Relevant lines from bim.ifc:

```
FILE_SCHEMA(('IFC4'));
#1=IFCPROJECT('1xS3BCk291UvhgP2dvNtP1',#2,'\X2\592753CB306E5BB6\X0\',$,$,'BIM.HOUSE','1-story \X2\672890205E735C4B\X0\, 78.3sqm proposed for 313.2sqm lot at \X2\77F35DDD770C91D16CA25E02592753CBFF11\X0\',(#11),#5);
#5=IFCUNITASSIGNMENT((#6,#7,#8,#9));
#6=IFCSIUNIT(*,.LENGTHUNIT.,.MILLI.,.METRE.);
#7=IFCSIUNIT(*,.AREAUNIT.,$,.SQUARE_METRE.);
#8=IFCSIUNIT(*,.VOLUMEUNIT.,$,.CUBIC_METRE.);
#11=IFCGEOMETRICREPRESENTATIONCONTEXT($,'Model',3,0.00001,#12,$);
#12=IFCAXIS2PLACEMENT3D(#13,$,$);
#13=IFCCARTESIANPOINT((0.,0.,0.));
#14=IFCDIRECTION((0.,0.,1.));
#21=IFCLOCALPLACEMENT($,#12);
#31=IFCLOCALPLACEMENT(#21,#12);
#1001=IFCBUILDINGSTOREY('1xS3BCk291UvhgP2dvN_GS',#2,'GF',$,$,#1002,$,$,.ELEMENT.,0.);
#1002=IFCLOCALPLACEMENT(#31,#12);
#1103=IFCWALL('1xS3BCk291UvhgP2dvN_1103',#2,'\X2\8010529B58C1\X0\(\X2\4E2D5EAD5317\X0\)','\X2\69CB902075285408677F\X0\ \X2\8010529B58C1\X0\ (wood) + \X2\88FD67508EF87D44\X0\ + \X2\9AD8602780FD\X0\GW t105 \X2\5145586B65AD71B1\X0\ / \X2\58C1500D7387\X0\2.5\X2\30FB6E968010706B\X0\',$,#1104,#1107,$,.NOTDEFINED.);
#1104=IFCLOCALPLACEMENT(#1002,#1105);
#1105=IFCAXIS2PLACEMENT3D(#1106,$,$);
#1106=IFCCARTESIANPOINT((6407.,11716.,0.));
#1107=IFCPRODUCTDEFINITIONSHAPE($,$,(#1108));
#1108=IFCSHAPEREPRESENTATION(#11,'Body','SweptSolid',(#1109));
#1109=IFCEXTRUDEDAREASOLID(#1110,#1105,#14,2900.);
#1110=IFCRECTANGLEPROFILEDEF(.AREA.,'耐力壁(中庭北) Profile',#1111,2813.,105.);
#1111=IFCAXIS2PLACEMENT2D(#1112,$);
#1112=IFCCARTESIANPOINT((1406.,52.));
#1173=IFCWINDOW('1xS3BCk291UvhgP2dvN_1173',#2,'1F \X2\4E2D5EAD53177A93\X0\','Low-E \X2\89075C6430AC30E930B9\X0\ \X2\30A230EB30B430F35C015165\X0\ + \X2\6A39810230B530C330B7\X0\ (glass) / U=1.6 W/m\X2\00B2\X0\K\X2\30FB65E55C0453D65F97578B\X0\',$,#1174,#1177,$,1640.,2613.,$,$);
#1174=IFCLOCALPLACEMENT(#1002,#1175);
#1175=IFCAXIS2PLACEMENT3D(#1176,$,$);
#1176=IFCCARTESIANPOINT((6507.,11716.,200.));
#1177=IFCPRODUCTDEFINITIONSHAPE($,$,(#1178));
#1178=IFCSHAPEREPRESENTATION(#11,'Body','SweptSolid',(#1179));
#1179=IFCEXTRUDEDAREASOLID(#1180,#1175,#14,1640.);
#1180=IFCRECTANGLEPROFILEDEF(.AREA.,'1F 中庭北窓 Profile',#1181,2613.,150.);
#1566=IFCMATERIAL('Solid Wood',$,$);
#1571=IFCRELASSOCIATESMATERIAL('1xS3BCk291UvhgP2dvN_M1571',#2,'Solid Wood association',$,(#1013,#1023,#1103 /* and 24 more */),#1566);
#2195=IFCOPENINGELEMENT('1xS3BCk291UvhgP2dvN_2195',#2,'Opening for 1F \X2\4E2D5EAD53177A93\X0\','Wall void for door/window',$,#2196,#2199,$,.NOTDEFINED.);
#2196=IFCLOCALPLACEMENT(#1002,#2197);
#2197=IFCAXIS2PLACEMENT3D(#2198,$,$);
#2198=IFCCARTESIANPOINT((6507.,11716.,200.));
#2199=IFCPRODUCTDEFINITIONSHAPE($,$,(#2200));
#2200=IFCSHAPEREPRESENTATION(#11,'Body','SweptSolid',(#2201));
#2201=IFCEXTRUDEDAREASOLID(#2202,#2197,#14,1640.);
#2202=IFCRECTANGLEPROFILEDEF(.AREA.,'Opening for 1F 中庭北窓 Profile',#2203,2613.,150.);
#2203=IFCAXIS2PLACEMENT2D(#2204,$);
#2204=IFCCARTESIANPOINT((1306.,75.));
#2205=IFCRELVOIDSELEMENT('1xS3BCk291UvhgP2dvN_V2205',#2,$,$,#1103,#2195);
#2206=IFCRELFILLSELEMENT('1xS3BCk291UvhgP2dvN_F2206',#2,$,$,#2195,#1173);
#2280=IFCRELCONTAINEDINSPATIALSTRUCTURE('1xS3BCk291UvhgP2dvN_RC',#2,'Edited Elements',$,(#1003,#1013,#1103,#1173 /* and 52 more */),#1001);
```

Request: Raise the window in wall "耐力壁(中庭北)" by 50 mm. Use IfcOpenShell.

```python
import numpy as np
import ifcopenshell
import ifcopenshell.api.geometry
import ifcopenshell.util.placement
import ifcopenshell.util.unit

model = ifcopenshell.open("bim.ifc")
unit_scale = ifcopenshell.util.unit.calculate_unit_scale(model)

window = model.by_guid("1xS3BCk291UvhgP2dvN_1173")
opening = window.FillsVoids[0].RelatingOpeningElement
dz = 0.05 / unit_scale

shift = np.array([0.0, 0.0, dz])
# The window is not placed relative to its opening, so move both.
for product in (opening, window):
    matrix = ifcopenshell.util.placement.get_local_placement(product.ObjectPlacement)
    matrix[:3, 3] += shift
    ifcopenshell.api.geometry.edit_object_placement(model, product=product, matrix=matrix, is_si=False)

print(f"moved by {dz * unit_scale:+.3f} m")

model.write("bim_updated.ifc")
```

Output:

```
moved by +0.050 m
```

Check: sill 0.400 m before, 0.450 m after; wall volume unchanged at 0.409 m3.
